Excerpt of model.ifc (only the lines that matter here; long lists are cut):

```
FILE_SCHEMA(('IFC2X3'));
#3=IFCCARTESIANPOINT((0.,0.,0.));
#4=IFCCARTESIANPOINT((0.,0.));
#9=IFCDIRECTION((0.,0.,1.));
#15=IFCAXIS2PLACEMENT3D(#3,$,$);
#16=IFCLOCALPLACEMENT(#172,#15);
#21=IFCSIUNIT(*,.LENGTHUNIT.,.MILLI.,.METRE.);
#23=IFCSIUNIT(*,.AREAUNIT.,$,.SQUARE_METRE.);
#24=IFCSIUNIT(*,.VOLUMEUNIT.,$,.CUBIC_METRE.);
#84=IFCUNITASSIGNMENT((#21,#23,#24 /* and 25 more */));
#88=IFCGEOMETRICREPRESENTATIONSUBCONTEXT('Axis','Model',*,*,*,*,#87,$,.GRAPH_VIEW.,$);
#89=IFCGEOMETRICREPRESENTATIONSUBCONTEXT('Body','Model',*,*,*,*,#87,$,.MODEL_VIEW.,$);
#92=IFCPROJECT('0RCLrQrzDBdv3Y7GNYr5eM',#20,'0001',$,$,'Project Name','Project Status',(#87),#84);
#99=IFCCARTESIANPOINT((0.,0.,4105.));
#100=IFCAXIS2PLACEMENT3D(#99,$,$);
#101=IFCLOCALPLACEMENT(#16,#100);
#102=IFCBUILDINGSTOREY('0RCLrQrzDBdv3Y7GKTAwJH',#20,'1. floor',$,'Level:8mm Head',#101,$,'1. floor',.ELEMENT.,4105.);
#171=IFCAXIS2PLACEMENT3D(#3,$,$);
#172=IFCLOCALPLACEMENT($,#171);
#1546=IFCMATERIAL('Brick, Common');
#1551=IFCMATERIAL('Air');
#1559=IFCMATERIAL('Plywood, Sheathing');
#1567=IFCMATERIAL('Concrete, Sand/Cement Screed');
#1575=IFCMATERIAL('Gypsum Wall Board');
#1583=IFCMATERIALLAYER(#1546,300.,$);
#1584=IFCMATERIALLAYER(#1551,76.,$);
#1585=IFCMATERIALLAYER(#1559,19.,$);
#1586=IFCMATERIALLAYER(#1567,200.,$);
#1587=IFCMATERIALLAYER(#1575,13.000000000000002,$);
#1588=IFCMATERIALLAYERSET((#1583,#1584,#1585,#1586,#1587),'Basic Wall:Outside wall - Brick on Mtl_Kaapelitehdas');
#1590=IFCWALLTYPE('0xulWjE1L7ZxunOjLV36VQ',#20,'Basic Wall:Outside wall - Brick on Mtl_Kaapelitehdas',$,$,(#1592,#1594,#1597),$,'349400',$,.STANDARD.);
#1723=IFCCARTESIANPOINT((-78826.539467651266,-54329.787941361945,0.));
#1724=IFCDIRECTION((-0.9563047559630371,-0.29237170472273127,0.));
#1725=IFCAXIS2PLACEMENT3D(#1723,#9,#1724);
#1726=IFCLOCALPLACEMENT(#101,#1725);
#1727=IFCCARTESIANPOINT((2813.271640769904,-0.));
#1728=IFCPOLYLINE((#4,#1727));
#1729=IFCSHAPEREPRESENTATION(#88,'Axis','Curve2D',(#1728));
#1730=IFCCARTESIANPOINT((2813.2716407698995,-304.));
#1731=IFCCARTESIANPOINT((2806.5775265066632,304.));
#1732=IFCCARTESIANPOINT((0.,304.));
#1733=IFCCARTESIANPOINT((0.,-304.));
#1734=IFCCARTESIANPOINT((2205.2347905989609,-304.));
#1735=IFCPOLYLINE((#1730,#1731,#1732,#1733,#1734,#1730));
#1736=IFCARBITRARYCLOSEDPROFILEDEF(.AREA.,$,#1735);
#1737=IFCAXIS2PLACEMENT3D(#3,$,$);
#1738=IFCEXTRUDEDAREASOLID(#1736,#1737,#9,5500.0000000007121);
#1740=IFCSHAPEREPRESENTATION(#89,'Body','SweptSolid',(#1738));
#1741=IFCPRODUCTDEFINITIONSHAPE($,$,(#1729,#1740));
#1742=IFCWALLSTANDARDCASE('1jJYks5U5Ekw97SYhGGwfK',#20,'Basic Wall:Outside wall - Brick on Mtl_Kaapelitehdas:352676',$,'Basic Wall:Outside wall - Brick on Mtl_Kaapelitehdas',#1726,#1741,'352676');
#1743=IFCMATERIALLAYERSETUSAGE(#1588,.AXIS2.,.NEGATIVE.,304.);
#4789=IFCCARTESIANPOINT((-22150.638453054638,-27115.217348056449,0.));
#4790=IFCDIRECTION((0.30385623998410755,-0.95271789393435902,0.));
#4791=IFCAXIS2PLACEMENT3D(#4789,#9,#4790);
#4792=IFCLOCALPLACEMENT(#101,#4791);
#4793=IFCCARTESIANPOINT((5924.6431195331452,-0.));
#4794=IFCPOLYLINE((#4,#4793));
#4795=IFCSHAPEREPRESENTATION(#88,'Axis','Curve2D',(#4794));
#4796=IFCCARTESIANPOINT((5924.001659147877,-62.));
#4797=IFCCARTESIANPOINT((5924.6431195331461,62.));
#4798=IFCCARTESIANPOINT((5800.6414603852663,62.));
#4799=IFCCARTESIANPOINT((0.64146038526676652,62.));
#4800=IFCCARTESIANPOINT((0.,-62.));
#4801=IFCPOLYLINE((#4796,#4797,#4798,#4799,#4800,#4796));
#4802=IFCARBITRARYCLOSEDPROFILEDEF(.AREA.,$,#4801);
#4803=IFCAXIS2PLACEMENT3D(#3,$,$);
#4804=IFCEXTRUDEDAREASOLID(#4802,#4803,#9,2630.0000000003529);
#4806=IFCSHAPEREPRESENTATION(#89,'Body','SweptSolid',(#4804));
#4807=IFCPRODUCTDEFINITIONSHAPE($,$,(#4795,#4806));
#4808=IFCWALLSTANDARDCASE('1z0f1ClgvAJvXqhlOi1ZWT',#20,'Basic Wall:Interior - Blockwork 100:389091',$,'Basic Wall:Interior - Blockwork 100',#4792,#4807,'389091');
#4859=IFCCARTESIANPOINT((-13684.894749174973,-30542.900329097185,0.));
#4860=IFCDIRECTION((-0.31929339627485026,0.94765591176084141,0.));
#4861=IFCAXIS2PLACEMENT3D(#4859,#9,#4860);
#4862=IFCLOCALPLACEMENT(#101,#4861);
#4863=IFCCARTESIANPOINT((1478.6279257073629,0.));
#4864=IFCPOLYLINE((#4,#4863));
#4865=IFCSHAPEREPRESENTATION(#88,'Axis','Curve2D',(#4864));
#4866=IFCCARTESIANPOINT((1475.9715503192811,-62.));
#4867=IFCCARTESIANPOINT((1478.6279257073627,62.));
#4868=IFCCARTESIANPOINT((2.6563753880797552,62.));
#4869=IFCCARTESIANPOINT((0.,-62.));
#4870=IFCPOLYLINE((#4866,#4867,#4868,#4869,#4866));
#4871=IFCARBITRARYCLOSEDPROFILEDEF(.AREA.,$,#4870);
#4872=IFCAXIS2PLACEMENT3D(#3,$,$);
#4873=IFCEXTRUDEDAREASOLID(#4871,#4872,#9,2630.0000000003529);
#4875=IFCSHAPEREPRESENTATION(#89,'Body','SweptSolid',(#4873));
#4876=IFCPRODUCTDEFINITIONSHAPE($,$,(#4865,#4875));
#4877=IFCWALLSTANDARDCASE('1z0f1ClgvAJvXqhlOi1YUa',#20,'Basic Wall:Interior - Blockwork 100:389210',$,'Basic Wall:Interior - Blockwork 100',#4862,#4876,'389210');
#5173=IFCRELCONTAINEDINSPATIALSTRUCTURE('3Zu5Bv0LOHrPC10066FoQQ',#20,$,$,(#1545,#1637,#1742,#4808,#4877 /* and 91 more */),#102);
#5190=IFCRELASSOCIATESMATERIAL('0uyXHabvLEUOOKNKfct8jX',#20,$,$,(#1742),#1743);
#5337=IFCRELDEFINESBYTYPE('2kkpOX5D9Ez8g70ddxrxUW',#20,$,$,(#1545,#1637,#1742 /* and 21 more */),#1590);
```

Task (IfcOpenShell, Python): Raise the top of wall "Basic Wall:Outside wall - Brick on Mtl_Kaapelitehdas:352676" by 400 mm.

```python
import ifcopenshell
import ifcopenshell.geom
import ifcopenshell.util.representation
import ifcopenshell.util.shape
import ifcopenshell.util.unit

model = ifcopenshell.open("model.ifc")
unit_scale = ifcopenshell.util.unit.calculate_unit_scale(model)
settings = ifcopenshell.geom.settings()


def volume(element):
    """Net volume in cubic metres, openings subtracted."""
    shape = ifcopenshell.geom.create_shape(settings, element)
    return ifcopenshell.util.shape.get_volume(shape.geometry)


wall = model.by_guid("1jJYks5U5Ekw97SYhGGwfK")
before = volume(wall)

body = ifcopenshell.util.representation.get_representation(wall, "Model", "Body")
solid = body.Items[0]
old_height = solid.Depth
solid.Depth += 0.4 / unit_scale
after = volume(wall)

print(f"height {old_height:g} -> {solid.Depth:g}, volume {before:.3f} -> {after:.3f} m3")

model.write("model-out.ifc")
```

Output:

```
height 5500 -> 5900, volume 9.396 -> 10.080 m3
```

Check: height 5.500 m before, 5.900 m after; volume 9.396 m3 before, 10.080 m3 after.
